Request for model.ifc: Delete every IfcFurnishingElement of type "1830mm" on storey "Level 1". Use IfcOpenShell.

First a look at what the model holds.

```python
import ifcopenshell
import ifcopenshell.util.element

model = ifcopenshell.open("model.ifc")
print(model.schema)
storey = next(s for s in model.by_type("IfcBuildingStorey") if s.Name == "Level 1")
furniture = [e for e in ifcopenshell.util.element.get_decomposition(storey) if e.is_a("IfcFurnishingElement")]
seen = {}
for e in furniture:
    element_type = ifcopenshell.util.element.get_type(e)
    name = element_type.Name if element_type not in (None, e) else None
    seen[name] = seen.get(name, 0) + 1
for name, count in sorted(seen.items(), key=str):
    print(count, "x", name)
```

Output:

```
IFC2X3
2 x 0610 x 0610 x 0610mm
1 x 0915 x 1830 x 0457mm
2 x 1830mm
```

```python
import ifcopenshell
import ifcopenshell.api.root
import ifcopenshell.util.element

model = ifcopenshell.open("model.ifc")

storey = next(s for s in model.by_type("IfcBuildingStorey") if s.Name == "Level 1")
furniture = [e for e in ifcopenshell.util.element.get_decomposition(storey) if e.is_a("IfcFurnishingElement")]
targets = [e for e in furniture if (t := ifcopenshell.util.element.get_type(e)) not in (None, e) and t.Name == "1830mm"]

for e in targets:
    ifcopenshell.api.root.remove_product(model, product=e)
print(len(targets), "removed")

model.write("model_v2.ifc")
```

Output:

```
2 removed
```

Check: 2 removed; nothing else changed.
